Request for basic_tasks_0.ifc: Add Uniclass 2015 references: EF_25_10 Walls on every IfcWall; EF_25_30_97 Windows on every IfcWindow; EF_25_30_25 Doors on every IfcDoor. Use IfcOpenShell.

First a look at what the model holds.

```python
import ifcopenshell

model = ifcopenshell.open("basic_tasks_0.ifc")
print(model.schema)
print("classifications:", [c.Name for c in model.by_type("IfcClassification")])
for ifc_class in ("IfcDoor", "IfcRoof", "IfcStair", "IfcWall", "IfcWindow"):
    print(ifc_class, len(model.by_type(ifc_class)))
```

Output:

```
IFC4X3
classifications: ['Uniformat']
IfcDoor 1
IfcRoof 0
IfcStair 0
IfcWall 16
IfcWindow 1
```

```python
import ifcopenshell
import ifcopenshell.api.classification

model = ifcopenshell.open("basic_tasks_0.ifc")

system = ifcopenshell.api.classification.add_classification(model, classification="Uniclass 2015")

codes = {
    "IfcWall": ("EF_25_10", "Walls"),
    "IfcWindow": ("EF_25_30_97", "Windows"),
    "IfcDoor": ("EF_25_30_25", "Doors"),
}
for ifc_class, (code, name) in codes.items():
    products = model.by_type(ifc_class)
    ifcopenshell.api.classification.add_reference(
        model, products=products, classification=system, identification=code, name=name
    )
    print(code, len(products))

model.write("basic_tasks_0_edited.ifc")
```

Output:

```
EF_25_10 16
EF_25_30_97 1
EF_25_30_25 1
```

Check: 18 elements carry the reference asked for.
